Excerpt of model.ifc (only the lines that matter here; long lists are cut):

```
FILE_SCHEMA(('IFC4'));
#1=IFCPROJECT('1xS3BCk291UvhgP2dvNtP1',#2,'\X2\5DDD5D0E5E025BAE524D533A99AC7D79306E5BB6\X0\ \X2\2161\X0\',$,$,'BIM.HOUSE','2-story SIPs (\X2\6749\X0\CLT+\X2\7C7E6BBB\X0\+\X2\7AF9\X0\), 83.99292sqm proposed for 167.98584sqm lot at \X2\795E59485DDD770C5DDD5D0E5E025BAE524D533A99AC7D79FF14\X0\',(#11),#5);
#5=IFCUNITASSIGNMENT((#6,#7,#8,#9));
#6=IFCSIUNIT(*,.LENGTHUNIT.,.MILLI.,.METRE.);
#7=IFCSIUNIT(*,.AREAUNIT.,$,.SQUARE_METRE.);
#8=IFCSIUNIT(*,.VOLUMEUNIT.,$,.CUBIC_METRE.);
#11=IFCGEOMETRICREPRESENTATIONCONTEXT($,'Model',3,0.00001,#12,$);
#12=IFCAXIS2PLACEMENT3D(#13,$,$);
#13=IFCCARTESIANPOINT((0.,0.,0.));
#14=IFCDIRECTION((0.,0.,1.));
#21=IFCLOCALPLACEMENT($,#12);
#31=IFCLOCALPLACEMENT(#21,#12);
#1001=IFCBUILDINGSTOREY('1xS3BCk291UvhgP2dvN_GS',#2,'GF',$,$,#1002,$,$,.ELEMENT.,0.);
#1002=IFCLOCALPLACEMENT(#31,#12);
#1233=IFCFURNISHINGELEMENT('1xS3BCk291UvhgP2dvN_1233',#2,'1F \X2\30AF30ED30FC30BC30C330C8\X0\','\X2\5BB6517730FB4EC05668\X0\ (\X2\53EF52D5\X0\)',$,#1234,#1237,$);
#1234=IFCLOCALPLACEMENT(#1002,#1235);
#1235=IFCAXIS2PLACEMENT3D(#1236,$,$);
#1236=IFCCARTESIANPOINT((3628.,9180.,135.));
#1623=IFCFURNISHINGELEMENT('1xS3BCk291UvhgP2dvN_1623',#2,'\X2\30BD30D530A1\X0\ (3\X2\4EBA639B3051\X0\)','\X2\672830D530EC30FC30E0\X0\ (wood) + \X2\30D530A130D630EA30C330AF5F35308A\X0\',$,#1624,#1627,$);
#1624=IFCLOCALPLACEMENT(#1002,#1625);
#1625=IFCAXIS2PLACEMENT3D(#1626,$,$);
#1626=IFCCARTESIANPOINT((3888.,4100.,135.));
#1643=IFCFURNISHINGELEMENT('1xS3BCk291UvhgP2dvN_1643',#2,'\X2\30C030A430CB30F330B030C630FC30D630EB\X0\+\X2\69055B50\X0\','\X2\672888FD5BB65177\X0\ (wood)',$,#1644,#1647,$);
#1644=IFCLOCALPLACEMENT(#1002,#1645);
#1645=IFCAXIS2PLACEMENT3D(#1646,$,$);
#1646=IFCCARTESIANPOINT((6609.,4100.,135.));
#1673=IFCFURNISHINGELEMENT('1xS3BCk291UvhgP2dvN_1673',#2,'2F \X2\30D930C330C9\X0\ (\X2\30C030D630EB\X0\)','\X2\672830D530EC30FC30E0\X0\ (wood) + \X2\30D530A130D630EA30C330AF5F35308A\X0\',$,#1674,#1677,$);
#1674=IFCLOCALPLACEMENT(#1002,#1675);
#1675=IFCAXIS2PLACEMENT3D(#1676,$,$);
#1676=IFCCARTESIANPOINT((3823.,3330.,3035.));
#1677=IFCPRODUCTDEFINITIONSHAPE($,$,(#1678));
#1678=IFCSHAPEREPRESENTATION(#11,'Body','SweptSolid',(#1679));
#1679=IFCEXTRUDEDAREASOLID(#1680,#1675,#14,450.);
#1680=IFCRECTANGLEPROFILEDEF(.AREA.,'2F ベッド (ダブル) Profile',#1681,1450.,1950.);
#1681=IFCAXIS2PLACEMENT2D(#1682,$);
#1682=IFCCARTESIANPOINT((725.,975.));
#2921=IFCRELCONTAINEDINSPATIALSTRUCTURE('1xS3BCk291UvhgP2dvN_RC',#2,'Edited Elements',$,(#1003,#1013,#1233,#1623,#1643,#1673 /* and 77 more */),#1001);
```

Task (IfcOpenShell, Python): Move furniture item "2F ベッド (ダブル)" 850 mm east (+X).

```python
import ifcopenshell
import ifcopenshell.api.geometry
import ifcopenshell.util.placement
import ifcopenshell.util.unit

model = ifcopenshell.open("model.ifc")
unit_scale = ifcopenshell.util.unit.calculate_unit_scale(model)

item = model.by_guid("1xS3BCk291UvhgP2dvN_1673")
matrix = ifcopenshell.util.placement.get_local_placement(item.ObjectPlacement)
matrix[0, 3] += 0.85 / unit_scale
ifcopenshell.api.geometry.edit_object_placement(model, product=item, matrix=matrix, is_si=False)

print(ifcopenshell.util.placement.get_local_placement(item.ObjectPlacement).round(3) + 0.0)

model.write("model-out.ifc")
```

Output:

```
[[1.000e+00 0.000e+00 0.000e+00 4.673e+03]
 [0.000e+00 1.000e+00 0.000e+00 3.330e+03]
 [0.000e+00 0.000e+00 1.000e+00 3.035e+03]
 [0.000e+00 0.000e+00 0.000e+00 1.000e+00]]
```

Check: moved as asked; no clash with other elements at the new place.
